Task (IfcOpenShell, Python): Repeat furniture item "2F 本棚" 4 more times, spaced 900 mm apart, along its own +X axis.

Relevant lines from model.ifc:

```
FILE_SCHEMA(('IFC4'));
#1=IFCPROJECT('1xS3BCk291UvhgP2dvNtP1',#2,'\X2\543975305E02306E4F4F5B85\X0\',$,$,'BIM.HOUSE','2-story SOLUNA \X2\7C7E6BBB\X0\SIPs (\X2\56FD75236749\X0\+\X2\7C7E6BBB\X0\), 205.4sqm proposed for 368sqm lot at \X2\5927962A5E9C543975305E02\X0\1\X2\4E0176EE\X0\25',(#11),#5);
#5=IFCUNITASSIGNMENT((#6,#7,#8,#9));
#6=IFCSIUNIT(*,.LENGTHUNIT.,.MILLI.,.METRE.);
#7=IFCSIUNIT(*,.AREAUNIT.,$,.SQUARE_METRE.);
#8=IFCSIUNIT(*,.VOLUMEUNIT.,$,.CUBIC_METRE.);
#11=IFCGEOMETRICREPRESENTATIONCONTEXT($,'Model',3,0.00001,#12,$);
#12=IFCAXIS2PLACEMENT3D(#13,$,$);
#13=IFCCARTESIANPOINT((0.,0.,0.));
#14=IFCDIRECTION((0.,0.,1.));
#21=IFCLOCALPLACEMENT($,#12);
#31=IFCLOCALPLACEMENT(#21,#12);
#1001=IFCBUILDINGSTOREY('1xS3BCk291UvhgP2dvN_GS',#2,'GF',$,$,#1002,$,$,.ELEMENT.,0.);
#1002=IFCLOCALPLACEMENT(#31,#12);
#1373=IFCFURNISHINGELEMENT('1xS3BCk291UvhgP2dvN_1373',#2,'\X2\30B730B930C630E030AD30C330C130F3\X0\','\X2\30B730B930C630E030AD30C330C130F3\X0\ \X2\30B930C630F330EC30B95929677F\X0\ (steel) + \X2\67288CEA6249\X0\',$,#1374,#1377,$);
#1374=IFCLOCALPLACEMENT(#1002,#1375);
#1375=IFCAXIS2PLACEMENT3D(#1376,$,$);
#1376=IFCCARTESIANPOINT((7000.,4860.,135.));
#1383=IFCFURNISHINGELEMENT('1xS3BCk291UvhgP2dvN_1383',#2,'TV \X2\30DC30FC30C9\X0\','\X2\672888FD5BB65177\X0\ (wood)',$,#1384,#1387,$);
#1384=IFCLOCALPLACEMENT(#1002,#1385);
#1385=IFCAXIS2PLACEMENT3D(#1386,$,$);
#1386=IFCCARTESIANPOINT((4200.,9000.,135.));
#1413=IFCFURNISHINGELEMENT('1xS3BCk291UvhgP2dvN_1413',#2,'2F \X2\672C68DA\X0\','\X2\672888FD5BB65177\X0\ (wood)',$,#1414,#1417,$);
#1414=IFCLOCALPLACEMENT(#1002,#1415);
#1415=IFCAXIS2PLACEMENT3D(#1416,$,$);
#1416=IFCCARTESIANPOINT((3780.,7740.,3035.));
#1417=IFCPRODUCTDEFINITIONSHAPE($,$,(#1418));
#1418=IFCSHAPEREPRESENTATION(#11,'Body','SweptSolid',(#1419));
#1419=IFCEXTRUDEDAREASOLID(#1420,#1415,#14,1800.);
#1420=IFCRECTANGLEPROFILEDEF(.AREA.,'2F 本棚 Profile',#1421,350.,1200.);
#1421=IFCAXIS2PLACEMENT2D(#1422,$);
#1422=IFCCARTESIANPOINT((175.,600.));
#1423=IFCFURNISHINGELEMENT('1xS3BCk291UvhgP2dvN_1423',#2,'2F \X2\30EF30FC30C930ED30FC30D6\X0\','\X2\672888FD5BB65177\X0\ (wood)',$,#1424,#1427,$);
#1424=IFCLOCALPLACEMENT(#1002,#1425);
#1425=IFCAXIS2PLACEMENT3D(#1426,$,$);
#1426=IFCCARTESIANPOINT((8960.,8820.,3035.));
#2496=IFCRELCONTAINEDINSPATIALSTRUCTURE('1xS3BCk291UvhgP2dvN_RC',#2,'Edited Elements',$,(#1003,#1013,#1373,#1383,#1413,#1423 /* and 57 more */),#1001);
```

```python
import ifcopenshell
import ifcopenshell.api.geometry
import ifcopenshell.api.root
import ifcopenshell.util.element
import ifcopenshell.util.placement

model = ifcopenshell.open("model.ifc")


def reuse_history(source, copy):
    """copy_class also copies each property set's owner history, people and application; keep the originals."""
    for rel in copy.IsDefinedBy:
        if rel.is_a("IfcRelDefinesByProperties") and (history := rel.RelatingPropertyDefinition.OwnerHistory):
            rel.RelatingPropertyDefinition.OwnerHistory = source.OwnerHistory
            ifcopenshell.util.element.remove_deep2(model, history)


source = model.by_guid("1xS3BCk291UvhgP2dvN_1413")
base = ifcopenshell.util.placement.get_local_placement(source.ObjectPlacement)
step = base[:3, 0] * 900.0

for i in range(1, 5):
    copy = ifcopenshell.api.root.copy_class(model, product=source)
    copy.Representation = ifcopenshell.util.element.copy_deep(
        model, source.Representation, exclude=["IfcGeometricRepresentationContext", "IfcRepresentationMap"]
    )
    reuse_history(source, copy)
    matrix = base.copy()
    matrix[:3, 3] += i * step
    print("added at", matrix[:3, 3].round(3) + 0.0)
    ifcopenshell.api.geometry.edit_object_placement(model, product=copy, matrix=matrix, is_si=False)

model.write("model_edited.ifc")
```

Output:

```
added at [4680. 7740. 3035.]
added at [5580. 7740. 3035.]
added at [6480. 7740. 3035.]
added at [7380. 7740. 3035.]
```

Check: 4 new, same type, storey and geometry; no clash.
